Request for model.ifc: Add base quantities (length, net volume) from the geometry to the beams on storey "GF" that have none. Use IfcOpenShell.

First a look at what the model holds.

```python
import ifcopenshell
import ifcopenshell.util.element
import ifcopenshell.util.unit

model = ifcopenshell.open("model.ifc")
print(model.schema)
for unit_type in ("LENGTHUNIT", "AREAUNIT", "VOLUMEUNIT"):
    print(unit_type, ifcopenshell.util.unit.calculate_unit_scale(model, unit_type))
storey = next(s for s in model.by_type("IfcBuildingStorey") if s.Name == "GF")
beams = [e for e in ifcopenshell.util.element.get_decomposition(storey) if e.is_a("IfcBeam")]
for e in sorted(beams, key=lambda e: e.id()):
    print(e.id(), e.is_a(), e.Name, list(ifcopenshell.util.element.get_psets(e, qtos_only=True)), sep=" | ")
```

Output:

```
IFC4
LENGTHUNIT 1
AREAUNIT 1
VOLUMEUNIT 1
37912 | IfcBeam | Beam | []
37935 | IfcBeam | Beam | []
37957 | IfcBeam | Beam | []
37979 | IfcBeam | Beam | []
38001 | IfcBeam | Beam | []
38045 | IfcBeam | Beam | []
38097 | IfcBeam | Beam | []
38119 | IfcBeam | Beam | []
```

```python
import ifcopenshell
import ifcopenshell.api.pset
import ifcopenshell.geom
import ifcopenshell.util.element
import ifcopenshell.util.shape
import ifcopenshell.util.unit

model = ifcopenshell.open("model.ifc")
unit_scale = ifcopenshell.util.unit.calculate_unit_scale(model)
volume_scale = ifcopenshell.util.unit.calculate_unit_scale(model, "VOLUMEUNIT")
settings = ifcopenshell.geom.settings()

storey = next(s for s in model.by_type("IfcBuildingStorey") if s.Name == "GF")
beams = [e for e in ifcopenshell.util.element.get_decomposition(storey) if e.is_a("IfcBeam")]

for e in sorted(beams, key=lambda e: e.id()):
    if ifcopenshell.util.element.get_psets(e, qtos_only=True, should_inherit=False):
        continue
    # Geometry comes back in metres, in the element's own axes.
    shape = ifcopenshell.geom.create_shape(settings, e)
    values = {
        "Length": ifcopenshell.util.shape.get_max_xyz(shape.geometry) / unit_scale,
        "NetVolume": ifcopenshell.util.shape.get_volume(shape.geometry) / volume_scale,
    }
    qto = ifcopenshell.api.pset.add_qto(model, product=e, name="Qto_BeamBaseQuantities")
    ifcopenshell.api.pset.edit_qto(model, qto=qto, properties=values)
    print(e.id(), {k: round(v, 3) for k, v in values.items()})

model.write("model-out.ifc")
```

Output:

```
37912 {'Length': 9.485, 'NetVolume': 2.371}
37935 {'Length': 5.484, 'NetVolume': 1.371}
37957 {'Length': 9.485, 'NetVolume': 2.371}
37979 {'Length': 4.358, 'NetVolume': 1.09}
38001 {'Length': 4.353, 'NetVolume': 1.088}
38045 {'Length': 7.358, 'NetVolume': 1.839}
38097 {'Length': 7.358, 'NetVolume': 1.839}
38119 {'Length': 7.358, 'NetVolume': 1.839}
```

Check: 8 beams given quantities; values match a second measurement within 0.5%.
